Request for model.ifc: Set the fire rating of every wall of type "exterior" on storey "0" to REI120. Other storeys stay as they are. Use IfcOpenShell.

First a look at what the model holds.

```python
import ifcopenshell
import ifcopenshell.util.element

model = ifcopenshell.open("model.ifc")
print(model.schema)
storey = next(s for s in model.by_type("IfcBuildingStorey") if s.Name == "0")
walls = [e for e in ifcopenshell.util.element.get_decomposition(storey) if e.is_a("IfcWall")]
seen = {}
for e in walls:
    element_type = ifcopenshell.util.element.get_type(e)
    key = (element_type.Name if element_type != e and element_type else None, ifcopenshell.util.element.get_pset(e, "Pset_WallCommon", "FireRating"))
    seen[key] = seen.get(key, 0) + 1
for (name, value), count in sorted(seen.items(), key=str):
    print(count, "x", name, "|", value)
```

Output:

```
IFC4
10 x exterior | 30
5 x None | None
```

```python
import ifcopenshell
import ifcopenshell.api.pset
import ifcopenshell.util.element

model = ifcopenshell.open("model.ifc")

storey = next(s for s in model.by_type("IfcBuildingStorey") if s.Name == "0")
walls = [e for e in ifcopenshell.util.element.get_decomposition(storey) if e.is_a("IfcWall")]

count = 0
for e in walls:
    element_type = ifcopenshell.util.element.get_type(e)
    if element_type in (None, e) or element_type.Name != "exterior":
        continue
    # add_pset returns the element's existing set when there is one.
    pset = ifcopenshell.api.pset.add_pset(model, product=e, name="Pset_WallCommon")
    ifcopenshell.api.pset.edit_pset(model, pset=pset, properties={"FireRating": "REI120"})
    count += 1

print(count, "walls updated")

model.write("model-out.ifc")
```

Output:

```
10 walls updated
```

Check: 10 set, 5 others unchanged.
